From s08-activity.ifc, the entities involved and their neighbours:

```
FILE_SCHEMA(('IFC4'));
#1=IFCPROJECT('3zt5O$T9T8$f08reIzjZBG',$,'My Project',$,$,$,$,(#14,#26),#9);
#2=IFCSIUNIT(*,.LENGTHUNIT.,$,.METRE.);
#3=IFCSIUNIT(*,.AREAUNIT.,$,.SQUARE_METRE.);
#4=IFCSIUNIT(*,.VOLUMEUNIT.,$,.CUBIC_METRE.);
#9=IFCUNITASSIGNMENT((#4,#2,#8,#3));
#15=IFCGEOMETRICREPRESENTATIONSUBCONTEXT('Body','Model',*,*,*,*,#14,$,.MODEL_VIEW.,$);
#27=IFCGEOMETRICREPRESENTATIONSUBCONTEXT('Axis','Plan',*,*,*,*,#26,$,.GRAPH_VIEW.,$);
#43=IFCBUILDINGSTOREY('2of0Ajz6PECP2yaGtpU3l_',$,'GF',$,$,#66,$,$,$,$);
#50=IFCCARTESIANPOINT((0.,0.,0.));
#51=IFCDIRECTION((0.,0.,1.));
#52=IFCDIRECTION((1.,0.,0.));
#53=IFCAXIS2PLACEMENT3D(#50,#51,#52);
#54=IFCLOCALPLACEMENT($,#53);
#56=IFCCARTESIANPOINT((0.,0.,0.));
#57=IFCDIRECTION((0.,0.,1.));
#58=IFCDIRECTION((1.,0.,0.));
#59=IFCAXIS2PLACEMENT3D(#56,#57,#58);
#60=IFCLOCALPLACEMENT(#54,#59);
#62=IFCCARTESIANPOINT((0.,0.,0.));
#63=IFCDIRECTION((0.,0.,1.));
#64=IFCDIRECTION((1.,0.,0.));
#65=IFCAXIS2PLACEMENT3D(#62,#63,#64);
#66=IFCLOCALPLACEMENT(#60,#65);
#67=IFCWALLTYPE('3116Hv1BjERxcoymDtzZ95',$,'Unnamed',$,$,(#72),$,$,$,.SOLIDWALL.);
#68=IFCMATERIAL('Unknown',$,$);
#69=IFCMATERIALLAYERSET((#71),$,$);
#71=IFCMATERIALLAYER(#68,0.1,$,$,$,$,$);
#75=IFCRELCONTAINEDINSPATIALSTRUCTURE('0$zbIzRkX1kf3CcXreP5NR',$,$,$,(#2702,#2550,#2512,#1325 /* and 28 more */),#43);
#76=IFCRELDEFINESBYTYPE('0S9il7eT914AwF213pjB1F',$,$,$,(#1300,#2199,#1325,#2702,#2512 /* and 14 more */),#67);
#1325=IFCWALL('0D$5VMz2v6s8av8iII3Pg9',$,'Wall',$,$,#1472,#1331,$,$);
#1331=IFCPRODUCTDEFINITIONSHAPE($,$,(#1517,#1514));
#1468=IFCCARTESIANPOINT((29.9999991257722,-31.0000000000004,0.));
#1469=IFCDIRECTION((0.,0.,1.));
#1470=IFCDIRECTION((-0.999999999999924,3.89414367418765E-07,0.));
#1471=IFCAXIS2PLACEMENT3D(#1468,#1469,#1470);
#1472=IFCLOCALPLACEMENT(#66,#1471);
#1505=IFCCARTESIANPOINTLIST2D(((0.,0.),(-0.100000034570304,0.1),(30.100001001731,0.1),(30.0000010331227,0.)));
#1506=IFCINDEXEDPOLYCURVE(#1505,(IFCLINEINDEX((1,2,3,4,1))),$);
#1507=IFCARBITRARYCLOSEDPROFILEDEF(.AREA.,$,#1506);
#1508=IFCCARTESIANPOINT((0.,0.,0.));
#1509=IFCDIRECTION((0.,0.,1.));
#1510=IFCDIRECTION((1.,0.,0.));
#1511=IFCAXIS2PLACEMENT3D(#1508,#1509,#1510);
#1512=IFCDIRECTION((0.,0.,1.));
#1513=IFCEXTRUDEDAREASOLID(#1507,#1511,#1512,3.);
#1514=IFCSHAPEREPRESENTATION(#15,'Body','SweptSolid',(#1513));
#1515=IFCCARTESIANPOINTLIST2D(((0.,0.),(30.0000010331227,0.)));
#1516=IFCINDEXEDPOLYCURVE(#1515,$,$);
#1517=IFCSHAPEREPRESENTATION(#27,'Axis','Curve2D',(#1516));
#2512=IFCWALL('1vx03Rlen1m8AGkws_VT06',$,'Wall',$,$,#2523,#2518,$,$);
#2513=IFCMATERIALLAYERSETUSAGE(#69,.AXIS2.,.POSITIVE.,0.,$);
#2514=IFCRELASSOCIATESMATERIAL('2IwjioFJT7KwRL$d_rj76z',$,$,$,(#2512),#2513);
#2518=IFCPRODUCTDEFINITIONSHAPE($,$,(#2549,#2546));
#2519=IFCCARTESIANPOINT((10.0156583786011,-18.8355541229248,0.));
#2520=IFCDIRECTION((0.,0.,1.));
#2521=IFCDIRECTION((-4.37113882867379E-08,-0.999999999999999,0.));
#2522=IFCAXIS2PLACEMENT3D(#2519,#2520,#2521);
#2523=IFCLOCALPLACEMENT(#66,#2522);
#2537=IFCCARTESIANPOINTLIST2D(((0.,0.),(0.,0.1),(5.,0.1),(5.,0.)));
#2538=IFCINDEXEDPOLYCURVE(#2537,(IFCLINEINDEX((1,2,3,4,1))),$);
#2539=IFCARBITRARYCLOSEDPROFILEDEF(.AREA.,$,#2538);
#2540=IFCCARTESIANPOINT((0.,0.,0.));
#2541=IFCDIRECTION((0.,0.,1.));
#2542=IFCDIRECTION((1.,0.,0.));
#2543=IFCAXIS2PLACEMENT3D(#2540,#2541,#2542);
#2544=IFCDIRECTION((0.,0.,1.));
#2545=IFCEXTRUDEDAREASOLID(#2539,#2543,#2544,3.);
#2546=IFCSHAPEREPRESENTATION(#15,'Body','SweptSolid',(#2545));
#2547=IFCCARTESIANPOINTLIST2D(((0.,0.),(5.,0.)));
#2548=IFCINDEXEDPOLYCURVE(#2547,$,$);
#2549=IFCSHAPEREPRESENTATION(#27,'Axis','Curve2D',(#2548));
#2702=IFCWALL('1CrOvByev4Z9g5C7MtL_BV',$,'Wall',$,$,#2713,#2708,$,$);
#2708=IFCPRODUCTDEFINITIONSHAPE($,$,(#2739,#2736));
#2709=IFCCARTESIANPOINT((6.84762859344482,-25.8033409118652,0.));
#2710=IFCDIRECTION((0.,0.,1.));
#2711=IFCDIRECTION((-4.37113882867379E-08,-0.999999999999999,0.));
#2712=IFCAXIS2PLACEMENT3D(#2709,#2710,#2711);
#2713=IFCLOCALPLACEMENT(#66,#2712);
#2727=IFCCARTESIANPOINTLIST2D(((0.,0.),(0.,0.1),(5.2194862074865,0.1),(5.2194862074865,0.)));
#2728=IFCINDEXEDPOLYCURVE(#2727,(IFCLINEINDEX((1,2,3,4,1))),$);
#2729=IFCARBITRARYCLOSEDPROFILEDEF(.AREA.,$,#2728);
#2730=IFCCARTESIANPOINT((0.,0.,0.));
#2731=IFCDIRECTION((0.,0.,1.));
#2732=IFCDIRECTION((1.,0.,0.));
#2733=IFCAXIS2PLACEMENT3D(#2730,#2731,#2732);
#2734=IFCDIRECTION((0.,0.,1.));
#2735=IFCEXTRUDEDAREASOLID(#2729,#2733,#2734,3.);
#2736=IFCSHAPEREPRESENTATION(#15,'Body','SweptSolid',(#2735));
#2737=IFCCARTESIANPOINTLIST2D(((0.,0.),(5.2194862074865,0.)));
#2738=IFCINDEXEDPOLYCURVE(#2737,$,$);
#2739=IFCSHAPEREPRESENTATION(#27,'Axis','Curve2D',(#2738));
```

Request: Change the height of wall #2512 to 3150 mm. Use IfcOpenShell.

```python
import ifcopenshell
import ifcopenshell.geom
import ifcopenshell.util.representation
import ifcopenshell.util.shape
import ifcopenshell.util.unit

model = ifcopenshell.open("s08-activity.ifc")
unit_scale = ifcopenshell.util.unit.calculate_unit_scale(model)
settings = ifcopenshell.geom.settings()


def volume(element):
    """Net volume in cubic metres, openings subtracted."""
    shape = ifcopenshell.geom.create_shape(settings, element)
    return ifcopenshell.util.shape.get_volume(shape.geometry)


wall = model.by_guid("1vx03Rlen1m8AGkws_VT06")
before = volume(wall)

body = ifcopenshell.util.representation.get_representation(wall, "Model", "Body")
solid = body.Items[0]
old_height = solid.Depth
solid.Depth = 3.15 / unit_scale
after = volume(wall)

print(f"height {old_height:g} -> {solid.Depth:g}, volume {before:.3f} -> {after:.3f} m3")

model.write("s08-activity_updated.ifc")
```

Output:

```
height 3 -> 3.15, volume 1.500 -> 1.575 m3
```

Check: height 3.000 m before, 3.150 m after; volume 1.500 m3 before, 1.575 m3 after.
